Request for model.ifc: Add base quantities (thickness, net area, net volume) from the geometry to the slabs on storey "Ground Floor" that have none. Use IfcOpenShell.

First a look at what the model holds.

```python
import ifcopenshell
import ifcopenshell.util.element
import ifcopenshell.util.unit

model = ifcopenshell.open("model.ifc")
print(model.schema)
for unit_type in ("LENGTHUNIT", "AREAUNIT", "VOLUMEUNIT"):
    print(unit_type, ifcopenshell.util.unit.calculate_unit_scale(model, unit_type))
storey = next(s for s in model.by_type("IfcBuildingStorey") if s.Name == "Ground Floor")
slabs = [e for e in ifcopenshell.util.element.get_decomposition(storey) if e.is_a("IfcSlab")]
for e in sorted(slabs, key=lambda e: e.id()):
    print(e.id(), e.is_a(), e.Name, list(ifcopenshell.util.element.get_psets(e, qtos_only=True)), sep=" | ")
```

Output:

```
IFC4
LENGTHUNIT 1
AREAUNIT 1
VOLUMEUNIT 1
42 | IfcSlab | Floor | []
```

```python
import ifcopenshell
import ifcopenshell.api.pset
import ifcopenshell.geom
import ifcopenshell.util.element
import ifcopenshell.util.shape
import ifcopenshell.util.unit

model = ifcopenshell.open("model.ifc")
unit_scale = ifcopenshell.util.unit.calculate_unit_scale(model)
area_scale = ifcopenshell.util.unit.calculate_unit_scale(model, "AREAUNIT")
volume_scale = ifcopenshell.util.unit.calculate_unit_scale(model, "VOLUMEUNIT")
settings = ifcopenshell.geom.settings()

storey = next(s for s in model.by_type("IfcBuildingStorey") if s.Name == "Ground Floor")
slabs = [e for e in ifcopenshell.util.element.get_decomposition(storey) if e.is_a("IfcSlab")]

for e in sorted(slabs, key=lambda e: e.id()):
    if ifcopenshell.util.element.get_psets(e, qtos_only=True, should_inherit=False):
        continue
    # Geometry comes back in metres, in the element's own axes.
    shape = ifcopenshell.geom.create_shape(settings, e)
    values = {
        "Width": ifcopenshell.util.shape.get_z(shape.geometry) / unit_scale,
        "NetArea": ifcopenshell.util.shape.get_footprint_area(shape.geometry) / area_scale,
        "NetVolume": ifcopenshell.util.shape.get_volume(shape.geometry) / volume_scale,
    }
    qto = ifcopenshell.api.pset.add_qto(model, product=e, name="Qto_SlabBaseQuantities")
    ifcopenshell.api.pset.edit_qto(model, qto=qto, properties=values)
    print(e.id(), {k: round(v, 3) for k, v in values.items()})

model.write("model_updated.ifc")
```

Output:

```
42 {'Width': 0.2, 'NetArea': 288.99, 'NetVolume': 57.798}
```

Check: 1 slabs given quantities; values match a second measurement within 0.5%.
